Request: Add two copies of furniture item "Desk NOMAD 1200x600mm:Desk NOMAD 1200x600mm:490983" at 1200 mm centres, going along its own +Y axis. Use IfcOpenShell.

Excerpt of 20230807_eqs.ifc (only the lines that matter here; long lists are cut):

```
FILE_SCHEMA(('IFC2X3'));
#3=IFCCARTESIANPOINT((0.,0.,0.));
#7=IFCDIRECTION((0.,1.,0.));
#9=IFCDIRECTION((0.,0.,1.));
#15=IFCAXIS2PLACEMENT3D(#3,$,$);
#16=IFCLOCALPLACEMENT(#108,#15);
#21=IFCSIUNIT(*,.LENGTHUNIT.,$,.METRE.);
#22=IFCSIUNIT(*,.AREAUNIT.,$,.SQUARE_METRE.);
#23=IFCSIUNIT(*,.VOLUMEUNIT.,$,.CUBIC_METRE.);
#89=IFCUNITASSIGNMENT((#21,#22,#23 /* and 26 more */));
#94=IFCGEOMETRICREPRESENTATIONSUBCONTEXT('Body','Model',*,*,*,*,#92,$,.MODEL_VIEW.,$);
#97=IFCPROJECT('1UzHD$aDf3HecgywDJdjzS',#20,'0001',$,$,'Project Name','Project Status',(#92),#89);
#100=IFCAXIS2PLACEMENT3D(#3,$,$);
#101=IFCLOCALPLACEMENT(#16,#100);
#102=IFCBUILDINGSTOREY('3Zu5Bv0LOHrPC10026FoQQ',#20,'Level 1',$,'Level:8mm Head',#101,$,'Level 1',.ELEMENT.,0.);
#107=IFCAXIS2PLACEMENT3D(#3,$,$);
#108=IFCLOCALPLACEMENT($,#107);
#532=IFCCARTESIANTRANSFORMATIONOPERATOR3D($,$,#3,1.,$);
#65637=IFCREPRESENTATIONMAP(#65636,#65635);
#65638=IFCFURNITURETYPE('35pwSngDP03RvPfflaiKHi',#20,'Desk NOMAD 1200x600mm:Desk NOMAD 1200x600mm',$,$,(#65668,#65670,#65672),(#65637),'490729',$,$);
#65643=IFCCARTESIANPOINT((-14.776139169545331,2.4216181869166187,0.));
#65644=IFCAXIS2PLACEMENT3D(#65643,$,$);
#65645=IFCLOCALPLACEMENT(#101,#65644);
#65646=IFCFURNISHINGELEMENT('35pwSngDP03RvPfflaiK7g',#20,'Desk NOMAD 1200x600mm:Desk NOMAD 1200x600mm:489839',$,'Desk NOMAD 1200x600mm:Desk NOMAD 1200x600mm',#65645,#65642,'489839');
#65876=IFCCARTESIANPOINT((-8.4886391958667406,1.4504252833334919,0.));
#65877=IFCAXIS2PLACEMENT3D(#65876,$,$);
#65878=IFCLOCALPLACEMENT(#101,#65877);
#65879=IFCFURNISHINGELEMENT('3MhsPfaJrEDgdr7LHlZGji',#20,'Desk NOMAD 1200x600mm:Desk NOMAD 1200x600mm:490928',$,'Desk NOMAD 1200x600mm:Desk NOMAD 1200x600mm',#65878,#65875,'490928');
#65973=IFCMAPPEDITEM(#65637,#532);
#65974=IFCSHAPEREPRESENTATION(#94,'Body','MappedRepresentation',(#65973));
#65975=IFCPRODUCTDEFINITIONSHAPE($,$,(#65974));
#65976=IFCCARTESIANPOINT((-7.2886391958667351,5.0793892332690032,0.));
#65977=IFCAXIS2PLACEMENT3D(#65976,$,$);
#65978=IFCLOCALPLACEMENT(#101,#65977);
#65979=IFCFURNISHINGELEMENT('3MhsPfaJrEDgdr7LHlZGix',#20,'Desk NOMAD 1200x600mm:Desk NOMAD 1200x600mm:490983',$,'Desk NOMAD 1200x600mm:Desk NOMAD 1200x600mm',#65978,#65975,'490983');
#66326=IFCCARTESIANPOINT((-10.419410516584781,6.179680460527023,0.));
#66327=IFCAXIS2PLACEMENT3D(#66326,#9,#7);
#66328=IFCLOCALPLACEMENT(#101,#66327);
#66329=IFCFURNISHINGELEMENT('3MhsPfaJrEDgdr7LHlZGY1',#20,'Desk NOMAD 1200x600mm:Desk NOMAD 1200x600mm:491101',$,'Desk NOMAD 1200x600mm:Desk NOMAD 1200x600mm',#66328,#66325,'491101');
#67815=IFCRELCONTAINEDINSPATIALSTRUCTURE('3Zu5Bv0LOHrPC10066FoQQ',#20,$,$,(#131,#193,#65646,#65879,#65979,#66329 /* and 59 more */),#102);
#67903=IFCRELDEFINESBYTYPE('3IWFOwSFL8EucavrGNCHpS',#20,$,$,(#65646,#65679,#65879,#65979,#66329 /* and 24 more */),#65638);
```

```python
import ifcopenshell
import ifcopenshell.api.geometry
import ifcopenshell.api.root
import ifcopenshell.util.element
import ifcopenshell.util.placement

model = ifcopenshell.open("20230807_eqs.ifc")


def reuse_history(source, copy):
    """copy_class also copies each property set's owner history, people and application; keep the originals."""
    for rel in copy.IsDefinedBy:
        if rel.is_a("IfcRelDefinesByProperties") and (history := rel.RelatingPropertyDefinition.OwnerHistory):
            rel.RelatingPropertyDefinition.OwnerHistory = source.OwnerHistory
            ifcopenshell.util.element.remove_deep2(model, history)


source = model.by_guid("3MhsPfaJrEDgdr7LHlZGix")
base = ifcopenshell.util.placement.get_local_placement(source.ObjectPlacement)
step = base[:3, 1] * 1.2

for i in range(1, 3):
    copy = ifcopenshell.api.root.copy_class(model, product=source)
    copy.Representation = ifcopenshell.util.element.copy_deep(
        model, source.Representation, exclude=["IfcGeometricRepresentationContext", "IfcRepresentationMap"]
    )
    copy.Name = "Desk NOMAD 1200x600mm:Desk NOMAD 1200x600mm"
    copy.Tag = None
    reuse_history(source, copy)
    matrix = base.copy()
    matrix[:3, 3] += i * step
    print("added at", matrix[:3, 3].round(3) + 0.0)
    ifcopenshell.api.geometry.edit_object_placement(model, product=copy, matrix=matrix, is_si=False)

model.write("20230807_eqs_rev.ifc")
```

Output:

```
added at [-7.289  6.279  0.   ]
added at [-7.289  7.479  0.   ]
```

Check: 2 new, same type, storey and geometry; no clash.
